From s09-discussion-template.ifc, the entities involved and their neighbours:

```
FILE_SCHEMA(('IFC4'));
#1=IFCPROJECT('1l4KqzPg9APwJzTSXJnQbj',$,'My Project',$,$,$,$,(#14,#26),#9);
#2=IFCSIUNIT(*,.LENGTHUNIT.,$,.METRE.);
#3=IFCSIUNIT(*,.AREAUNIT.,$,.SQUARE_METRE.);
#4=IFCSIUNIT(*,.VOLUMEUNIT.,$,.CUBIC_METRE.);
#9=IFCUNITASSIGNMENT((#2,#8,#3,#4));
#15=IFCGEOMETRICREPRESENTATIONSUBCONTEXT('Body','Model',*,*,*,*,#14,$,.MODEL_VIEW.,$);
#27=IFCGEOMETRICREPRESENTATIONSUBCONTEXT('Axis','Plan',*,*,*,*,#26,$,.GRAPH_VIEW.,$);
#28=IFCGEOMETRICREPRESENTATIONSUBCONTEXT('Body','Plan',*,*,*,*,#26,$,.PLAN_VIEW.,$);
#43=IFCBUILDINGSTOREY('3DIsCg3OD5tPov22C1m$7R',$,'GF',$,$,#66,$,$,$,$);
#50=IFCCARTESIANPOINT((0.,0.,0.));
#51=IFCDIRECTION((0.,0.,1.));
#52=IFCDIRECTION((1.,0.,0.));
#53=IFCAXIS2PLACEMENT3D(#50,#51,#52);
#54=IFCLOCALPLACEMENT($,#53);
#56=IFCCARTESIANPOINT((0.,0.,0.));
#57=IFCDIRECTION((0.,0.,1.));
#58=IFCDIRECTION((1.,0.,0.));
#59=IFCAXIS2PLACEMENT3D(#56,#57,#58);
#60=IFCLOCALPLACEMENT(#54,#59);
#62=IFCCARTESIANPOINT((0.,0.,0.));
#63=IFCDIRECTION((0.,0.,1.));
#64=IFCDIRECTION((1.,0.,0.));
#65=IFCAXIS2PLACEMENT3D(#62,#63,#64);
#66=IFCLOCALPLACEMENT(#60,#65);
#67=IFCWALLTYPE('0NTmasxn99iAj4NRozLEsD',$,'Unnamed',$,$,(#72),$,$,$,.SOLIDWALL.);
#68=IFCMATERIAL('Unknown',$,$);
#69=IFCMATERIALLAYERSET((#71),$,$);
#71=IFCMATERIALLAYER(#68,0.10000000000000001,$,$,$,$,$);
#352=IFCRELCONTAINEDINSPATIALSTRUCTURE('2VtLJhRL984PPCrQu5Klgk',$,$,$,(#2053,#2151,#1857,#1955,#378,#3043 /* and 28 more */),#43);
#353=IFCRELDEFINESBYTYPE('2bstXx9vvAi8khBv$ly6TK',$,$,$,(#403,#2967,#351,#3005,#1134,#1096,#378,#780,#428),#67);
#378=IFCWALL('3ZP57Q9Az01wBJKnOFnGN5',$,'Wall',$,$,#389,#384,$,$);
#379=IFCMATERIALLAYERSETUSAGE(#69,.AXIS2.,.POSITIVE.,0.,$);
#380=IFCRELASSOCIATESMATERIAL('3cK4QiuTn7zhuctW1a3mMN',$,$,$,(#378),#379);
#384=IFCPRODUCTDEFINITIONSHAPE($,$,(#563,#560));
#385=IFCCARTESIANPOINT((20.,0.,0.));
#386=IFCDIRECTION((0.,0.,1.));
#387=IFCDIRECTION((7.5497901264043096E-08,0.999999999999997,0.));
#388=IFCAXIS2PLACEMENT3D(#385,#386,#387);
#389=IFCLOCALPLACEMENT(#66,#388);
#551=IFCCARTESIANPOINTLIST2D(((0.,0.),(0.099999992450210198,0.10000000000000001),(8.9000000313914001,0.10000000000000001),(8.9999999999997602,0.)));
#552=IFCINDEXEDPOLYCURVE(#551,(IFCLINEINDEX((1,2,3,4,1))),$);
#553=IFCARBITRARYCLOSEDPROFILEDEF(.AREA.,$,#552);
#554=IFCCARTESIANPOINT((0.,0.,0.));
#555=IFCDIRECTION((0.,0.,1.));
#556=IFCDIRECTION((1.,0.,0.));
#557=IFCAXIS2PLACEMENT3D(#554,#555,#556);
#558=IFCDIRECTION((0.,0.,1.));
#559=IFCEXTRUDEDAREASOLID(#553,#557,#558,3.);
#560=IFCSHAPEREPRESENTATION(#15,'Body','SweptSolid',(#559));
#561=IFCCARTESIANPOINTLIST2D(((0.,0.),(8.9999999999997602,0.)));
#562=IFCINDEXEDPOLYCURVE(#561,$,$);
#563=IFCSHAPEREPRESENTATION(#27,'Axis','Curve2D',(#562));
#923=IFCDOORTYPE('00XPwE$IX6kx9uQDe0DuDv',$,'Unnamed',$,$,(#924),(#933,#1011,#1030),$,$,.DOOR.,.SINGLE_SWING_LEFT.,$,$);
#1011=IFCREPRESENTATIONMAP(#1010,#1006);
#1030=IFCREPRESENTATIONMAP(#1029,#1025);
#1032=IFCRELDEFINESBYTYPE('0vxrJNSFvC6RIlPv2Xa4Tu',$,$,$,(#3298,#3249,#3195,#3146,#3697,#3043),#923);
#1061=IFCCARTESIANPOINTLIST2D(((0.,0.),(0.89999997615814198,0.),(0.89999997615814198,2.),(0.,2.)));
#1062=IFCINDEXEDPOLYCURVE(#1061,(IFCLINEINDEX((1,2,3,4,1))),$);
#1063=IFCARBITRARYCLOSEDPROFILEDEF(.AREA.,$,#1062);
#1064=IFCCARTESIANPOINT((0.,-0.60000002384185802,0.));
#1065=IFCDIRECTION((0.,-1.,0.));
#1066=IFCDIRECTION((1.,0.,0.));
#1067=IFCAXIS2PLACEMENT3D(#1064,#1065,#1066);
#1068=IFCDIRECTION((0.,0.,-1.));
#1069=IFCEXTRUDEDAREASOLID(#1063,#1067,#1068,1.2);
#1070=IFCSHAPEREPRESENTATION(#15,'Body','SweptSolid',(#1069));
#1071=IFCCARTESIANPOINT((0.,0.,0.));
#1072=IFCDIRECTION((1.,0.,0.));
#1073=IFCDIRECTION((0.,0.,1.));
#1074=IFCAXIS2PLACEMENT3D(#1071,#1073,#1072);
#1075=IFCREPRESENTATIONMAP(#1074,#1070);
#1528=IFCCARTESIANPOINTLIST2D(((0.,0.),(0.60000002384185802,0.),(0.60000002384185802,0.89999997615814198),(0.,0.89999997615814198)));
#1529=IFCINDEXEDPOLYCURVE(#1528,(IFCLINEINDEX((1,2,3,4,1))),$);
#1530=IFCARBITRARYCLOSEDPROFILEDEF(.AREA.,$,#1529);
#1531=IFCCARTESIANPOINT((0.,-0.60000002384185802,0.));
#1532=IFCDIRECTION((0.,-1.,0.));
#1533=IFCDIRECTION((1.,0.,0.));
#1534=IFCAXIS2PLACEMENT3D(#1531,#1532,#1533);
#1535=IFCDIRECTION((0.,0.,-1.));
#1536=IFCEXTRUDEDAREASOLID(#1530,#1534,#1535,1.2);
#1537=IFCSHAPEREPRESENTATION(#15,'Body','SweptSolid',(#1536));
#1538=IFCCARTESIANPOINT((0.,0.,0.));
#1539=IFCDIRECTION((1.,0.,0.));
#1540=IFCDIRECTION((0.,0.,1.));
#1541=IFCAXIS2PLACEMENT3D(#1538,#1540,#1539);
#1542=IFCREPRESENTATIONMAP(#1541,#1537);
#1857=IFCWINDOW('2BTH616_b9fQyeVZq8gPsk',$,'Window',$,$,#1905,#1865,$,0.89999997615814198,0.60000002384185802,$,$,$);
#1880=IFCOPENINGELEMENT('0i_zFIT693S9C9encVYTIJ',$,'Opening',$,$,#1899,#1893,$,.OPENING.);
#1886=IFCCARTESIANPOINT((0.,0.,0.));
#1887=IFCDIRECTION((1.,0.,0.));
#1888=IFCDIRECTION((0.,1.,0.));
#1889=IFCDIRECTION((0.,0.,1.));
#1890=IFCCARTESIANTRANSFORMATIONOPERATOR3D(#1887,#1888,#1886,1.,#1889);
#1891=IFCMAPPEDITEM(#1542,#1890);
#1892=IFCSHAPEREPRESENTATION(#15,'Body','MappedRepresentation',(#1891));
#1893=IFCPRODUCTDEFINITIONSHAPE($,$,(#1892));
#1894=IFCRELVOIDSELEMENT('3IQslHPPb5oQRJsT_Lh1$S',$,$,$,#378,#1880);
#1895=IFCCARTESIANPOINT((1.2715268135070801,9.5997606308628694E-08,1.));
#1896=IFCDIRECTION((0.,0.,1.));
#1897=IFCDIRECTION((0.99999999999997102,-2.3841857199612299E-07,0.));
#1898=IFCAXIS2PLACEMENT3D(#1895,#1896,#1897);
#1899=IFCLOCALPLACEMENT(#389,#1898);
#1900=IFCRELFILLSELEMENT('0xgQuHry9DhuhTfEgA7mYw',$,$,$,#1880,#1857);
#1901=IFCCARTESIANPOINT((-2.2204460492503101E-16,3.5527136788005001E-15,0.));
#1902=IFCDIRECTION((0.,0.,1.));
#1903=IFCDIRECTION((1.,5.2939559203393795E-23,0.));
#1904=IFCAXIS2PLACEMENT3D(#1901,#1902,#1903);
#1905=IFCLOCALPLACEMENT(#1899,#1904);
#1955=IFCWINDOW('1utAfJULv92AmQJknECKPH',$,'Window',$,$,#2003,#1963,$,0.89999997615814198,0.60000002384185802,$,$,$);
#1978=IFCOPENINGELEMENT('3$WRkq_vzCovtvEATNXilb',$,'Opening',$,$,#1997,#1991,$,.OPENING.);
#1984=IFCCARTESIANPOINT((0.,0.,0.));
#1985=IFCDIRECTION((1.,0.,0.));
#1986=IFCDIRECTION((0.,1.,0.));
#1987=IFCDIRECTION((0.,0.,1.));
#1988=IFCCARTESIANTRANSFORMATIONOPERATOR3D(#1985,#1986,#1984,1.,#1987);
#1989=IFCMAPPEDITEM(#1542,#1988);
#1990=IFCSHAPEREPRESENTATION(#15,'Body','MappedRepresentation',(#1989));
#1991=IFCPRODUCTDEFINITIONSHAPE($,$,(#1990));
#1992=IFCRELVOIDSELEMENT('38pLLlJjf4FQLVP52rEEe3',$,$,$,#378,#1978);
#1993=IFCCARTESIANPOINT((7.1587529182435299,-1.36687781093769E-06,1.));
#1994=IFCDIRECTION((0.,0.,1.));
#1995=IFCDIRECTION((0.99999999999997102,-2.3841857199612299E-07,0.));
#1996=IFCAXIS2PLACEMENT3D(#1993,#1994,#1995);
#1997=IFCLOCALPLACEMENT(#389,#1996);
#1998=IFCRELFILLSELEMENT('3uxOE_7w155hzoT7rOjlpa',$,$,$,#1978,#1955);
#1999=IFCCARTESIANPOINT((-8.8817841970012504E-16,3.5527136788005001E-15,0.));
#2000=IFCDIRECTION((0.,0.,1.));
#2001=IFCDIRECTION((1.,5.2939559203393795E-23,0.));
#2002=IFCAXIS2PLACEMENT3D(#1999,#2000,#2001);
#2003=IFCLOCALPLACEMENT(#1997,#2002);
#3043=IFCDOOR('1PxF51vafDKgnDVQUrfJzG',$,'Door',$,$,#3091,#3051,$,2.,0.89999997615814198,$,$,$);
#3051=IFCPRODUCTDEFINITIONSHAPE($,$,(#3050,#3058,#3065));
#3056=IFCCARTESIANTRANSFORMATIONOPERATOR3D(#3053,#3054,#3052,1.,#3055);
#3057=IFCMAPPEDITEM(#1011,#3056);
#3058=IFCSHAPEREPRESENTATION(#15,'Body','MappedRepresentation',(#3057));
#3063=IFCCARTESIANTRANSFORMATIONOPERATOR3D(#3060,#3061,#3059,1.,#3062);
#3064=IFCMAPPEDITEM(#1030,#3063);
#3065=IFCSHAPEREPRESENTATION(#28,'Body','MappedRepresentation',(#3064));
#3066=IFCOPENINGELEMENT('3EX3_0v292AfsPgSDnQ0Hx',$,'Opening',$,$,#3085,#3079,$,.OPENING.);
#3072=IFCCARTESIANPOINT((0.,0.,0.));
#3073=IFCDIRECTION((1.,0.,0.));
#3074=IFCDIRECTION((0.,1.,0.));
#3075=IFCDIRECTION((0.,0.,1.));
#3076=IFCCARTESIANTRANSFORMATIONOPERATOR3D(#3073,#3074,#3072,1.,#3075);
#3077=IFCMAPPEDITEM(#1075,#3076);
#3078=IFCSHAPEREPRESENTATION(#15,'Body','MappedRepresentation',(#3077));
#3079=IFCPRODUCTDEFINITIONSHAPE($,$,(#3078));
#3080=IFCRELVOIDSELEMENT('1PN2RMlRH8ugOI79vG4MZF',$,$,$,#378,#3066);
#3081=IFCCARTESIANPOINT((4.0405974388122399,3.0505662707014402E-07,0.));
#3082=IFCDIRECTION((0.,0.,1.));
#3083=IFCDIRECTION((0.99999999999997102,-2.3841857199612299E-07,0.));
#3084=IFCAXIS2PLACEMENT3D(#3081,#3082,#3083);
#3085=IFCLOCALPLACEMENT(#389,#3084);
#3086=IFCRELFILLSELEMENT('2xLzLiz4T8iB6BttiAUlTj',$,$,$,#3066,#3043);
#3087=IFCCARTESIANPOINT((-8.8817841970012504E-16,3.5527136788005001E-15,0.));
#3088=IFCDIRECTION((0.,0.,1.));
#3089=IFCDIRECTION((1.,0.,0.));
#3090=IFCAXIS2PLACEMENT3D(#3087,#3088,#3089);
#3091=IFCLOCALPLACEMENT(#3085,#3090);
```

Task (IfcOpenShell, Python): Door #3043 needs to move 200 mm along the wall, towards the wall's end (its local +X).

```python
import ifcopenshell
import ifcopenshell.api.geometry
import ifcopenshell.util.placement

model = ifcopenshell.open("s09-discussion-template.ifc")

door = model.by_guid("1PxF51vafDKgnDVQUrfJzG")
opening = door.FillsVoids[0].RelatingOpeningElement
wall = opening.VoidsElements[0].RelatingBuildingElement

wall_matrix = ifcopenshell.util.placement.get_local_placement(wall.ObjectPlacement)
shift = wall_matrix[:3, 0] * 0.2
before = ifcopenshell.util.placement.get_local_placement(door.ObjectPlacement)[:3, 3].copy()

# The door is placed relative to its opening, so it follows when the opening moves.
matrix = ifcopenshell.util.placement.get_local_placement(opening.ObjectPlacement)
matrix[:3, 3] += shift
ifcopenshell.api.geometry.edit_object_placement(
    model, product=opening, matrix=matrix, is_si=False, should_transform_children=True
)

after = ifcopenshell.util.placement.get_local_placement(door.ObjectPlacement)[:3, 3]
print("door moved by", (after - before).round(3) + 0.0)

model.write("s09-discussion-template_edited.ifc")
```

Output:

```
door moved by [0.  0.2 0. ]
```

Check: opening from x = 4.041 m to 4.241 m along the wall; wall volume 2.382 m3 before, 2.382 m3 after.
